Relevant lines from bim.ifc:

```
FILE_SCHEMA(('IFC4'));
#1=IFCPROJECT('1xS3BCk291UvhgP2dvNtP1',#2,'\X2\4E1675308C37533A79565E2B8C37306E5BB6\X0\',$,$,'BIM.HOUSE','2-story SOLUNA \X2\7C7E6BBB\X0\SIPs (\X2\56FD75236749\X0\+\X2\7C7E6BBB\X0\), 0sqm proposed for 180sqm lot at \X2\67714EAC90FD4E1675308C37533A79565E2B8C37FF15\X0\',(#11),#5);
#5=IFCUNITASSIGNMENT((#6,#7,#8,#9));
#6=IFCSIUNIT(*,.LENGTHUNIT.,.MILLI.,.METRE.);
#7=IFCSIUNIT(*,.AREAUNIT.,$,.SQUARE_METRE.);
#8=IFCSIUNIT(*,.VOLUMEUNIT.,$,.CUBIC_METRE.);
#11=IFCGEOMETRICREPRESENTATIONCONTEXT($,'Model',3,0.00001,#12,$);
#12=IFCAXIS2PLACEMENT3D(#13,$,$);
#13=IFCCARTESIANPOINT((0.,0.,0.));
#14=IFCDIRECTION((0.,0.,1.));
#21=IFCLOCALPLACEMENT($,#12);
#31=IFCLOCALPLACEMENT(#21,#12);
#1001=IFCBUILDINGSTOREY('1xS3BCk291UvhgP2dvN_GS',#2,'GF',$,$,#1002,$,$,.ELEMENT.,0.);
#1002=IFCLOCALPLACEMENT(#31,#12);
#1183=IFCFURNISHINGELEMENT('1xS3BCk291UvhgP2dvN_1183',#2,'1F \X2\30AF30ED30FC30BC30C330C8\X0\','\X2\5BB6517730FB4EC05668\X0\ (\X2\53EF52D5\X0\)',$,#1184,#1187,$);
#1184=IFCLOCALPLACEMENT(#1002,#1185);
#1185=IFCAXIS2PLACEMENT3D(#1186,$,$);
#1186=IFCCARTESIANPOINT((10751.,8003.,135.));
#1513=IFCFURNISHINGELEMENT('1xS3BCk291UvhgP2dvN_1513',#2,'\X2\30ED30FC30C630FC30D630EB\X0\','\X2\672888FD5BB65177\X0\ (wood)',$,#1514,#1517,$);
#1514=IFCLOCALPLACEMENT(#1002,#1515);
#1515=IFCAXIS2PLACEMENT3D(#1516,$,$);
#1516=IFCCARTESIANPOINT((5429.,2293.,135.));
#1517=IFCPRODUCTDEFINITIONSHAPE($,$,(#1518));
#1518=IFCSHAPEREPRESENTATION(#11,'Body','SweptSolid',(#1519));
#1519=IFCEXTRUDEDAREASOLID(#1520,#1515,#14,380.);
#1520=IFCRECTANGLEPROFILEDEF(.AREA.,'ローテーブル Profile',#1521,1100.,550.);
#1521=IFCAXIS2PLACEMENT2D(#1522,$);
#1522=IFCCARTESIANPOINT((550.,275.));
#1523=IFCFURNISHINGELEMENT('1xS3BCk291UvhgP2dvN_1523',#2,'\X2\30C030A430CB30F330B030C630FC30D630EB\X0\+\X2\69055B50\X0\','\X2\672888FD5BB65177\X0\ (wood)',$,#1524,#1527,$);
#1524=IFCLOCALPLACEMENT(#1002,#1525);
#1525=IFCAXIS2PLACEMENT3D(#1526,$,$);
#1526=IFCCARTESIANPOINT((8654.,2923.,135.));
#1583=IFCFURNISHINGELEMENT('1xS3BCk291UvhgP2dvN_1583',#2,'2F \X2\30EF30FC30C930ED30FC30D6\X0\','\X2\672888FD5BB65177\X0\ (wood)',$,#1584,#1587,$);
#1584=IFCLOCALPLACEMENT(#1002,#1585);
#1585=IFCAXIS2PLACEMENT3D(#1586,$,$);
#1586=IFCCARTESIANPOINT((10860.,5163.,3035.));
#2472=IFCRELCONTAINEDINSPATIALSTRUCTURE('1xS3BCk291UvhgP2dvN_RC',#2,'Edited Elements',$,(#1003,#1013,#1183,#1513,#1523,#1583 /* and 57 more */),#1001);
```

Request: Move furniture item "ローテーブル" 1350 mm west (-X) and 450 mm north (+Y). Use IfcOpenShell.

```python
import ifcopenshell
import ifcopenshell.api.geometry
import ifcopenshell.util.placement
import ifcopenshell.util.unit

model = ifcopenshell.open("bim.ifc")
unit_scale = ifcopenshell.util.unit.calculate_unit_scale(model)

item = model.by_id(1513)
matrix = ifcopenshell.util.placement.get_local_placement(item.ObjectPlacement)
matrix[0, 3] -= 1.35 / unit_scale
matrix[1, 3] += 0.45 / unit_scale
ifcopenshell.api.geometry.edit_object_placement(model, product=item, matrix=matrix, is_si=False)

print(ifcopenshell.util.placement.get_local_placement(item.ObjectPlacement).round(3) + 0.0)

model.write("bim_rev.ifc")
```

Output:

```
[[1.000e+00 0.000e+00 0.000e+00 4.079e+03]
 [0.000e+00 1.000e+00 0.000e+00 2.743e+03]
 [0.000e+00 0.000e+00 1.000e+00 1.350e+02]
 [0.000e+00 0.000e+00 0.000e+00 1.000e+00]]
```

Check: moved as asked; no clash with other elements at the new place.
